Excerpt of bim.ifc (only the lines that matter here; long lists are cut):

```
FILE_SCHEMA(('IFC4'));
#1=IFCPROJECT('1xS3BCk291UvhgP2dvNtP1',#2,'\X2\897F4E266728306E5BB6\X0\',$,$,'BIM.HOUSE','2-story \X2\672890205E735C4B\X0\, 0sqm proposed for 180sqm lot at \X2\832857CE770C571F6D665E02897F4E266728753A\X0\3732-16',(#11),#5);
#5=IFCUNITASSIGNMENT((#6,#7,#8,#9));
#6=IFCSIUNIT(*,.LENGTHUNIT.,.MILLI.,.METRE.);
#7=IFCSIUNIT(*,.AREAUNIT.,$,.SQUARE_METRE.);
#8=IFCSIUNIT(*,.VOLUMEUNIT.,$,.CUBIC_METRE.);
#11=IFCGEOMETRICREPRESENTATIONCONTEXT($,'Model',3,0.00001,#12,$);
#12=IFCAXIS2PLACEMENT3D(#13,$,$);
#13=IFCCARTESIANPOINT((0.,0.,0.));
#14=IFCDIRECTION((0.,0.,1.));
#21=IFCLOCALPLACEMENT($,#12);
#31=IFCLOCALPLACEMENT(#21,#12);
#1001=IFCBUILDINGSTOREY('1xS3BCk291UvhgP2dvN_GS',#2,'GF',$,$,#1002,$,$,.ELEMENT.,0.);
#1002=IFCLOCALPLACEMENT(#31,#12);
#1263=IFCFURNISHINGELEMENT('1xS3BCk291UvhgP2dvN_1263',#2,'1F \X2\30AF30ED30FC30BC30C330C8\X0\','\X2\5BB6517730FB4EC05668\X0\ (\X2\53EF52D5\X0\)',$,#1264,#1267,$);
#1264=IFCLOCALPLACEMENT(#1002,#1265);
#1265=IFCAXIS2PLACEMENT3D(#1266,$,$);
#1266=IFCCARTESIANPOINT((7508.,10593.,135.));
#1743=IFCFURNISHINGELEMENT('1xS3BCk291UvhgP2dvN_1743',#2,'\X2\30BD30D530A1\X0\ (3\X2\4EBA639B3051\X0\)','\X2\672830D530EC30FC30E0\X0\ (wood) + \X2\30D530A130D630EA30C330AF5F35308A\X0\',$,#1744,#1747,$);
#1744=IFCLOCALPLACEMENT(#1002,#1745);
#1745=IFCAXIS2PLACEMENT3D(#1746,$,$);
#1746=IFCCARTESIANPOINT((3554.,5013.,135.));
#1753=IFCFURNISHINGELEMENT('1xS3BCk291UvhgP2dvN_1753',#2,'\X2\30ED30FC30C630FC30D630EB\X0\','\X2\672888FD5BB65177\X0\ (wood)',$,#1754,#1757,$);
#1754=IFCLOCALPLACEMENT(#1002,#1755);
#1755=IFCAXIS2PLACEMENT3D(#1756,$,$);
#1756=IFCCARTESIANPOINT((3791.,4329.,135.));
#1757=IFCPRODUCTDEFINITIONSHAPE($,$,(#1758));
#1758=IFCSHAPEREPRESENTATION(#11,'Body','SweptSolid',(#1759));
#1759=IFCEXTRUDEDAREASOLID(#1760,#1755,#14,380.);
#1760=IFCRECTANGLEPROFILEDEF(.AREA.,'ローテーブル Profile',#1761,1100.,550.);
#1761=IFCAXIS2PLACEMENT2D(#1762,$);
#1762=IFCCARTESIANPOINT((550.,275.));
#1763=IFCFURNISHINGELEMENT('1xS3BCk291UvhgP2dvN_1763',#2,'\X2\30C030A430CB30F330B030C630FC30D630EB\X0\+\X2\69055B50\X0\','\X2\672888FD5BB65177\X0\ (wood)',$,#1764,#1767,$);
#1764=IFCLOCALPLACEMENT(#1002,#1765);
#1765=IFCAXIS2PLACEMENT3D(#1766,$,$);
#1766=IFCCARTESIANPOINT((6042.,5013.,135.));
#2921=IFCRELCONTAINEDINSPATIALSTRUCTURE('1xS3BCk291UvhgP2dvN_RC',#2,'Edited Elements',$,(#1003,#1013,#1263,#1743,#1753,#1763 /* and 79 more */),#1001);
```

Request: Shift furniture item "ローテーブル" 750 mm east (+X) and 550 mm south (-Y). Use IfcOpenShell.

```python
import ifcopenshell
import ifcopenshell.api.geometry
import ifcopenshell.util.placement
import ifcopenshell.util.unit

model = ifcopenshell.open("bim.ifc")
unit_scale = ifcopenshell.util.unit.calculate_unit_scale(model)

item = model.by_guid("1xS3BCk291UvhgP2dvN_1753")
matrix = ifcopenshell.util.placement.get_local_placement(item.ObjectPlacement)
matrix[0, 3] += 0.75 / unit_scale
matrix[1, 3] -= 0.55 / unit_scale
ifcopenshell.api.geometry.edit_object_placement(model, product=item, matrix=matrix, is_si=False)

print(ifcopenshell.util.placement.get_local_placement(item.ObjectPlacement).round(3) + 0.0)

model.write("bim_rev.ifc")
```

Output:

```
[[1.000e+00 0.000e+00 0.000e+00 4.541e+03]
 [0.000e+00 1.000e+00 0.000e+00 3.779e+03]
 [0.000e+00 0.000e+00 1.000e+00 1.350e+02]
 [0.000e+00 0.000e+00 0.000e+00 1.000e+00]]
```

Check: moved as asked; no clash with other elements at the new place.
